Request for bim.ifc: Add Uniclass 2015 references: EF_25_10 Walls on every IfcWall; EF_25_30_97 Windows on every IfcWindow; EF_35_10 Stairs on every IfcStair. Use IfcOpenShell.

First a look at what the model holds.

```python
import ifcopenshell

model = ifcopenshell.open("bim.ifc")
print(model.schema)
print("classifications:", [c.Name for c in model.by_type("IfcClassification")])
for ifc_class in ("IfcDoor", "IfcRoof", "IfcStair", "IfcWall", "IfcWindow"):
    print(ifc_class, len(model.by_type(ifc_class)))
```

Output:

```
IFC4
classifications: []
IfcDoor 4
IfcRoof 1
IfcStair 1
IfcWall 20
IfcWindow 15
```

```python
import ifcopenshell
import ifcopenshell.api.classification

model = ifcopenshell.open("bim.ifc")

system = ifcopenshell.api.classification.add_classification(model, classification="Uniclass 2015")

codes = {
    "IfcWall": ("EF_25_10", "Walls"),
    "IfcWindow": ("EF_25_30_97", "Windows"),
    "IfcStair": ("EF_35_10", "Stairs"),
}
for ifc_class, (code, name) in codes.items():
    products = model.by_type(ifc_class)
    ifcopenshell.api.classification.add_reference(
        model, products=products, classification=system, identification=code, name=name
    )
    print(code, len(products))

model.write("bim_edited.ifc")
```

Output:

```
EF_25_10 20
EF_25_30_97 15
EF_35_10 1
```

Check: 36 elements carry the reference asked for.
